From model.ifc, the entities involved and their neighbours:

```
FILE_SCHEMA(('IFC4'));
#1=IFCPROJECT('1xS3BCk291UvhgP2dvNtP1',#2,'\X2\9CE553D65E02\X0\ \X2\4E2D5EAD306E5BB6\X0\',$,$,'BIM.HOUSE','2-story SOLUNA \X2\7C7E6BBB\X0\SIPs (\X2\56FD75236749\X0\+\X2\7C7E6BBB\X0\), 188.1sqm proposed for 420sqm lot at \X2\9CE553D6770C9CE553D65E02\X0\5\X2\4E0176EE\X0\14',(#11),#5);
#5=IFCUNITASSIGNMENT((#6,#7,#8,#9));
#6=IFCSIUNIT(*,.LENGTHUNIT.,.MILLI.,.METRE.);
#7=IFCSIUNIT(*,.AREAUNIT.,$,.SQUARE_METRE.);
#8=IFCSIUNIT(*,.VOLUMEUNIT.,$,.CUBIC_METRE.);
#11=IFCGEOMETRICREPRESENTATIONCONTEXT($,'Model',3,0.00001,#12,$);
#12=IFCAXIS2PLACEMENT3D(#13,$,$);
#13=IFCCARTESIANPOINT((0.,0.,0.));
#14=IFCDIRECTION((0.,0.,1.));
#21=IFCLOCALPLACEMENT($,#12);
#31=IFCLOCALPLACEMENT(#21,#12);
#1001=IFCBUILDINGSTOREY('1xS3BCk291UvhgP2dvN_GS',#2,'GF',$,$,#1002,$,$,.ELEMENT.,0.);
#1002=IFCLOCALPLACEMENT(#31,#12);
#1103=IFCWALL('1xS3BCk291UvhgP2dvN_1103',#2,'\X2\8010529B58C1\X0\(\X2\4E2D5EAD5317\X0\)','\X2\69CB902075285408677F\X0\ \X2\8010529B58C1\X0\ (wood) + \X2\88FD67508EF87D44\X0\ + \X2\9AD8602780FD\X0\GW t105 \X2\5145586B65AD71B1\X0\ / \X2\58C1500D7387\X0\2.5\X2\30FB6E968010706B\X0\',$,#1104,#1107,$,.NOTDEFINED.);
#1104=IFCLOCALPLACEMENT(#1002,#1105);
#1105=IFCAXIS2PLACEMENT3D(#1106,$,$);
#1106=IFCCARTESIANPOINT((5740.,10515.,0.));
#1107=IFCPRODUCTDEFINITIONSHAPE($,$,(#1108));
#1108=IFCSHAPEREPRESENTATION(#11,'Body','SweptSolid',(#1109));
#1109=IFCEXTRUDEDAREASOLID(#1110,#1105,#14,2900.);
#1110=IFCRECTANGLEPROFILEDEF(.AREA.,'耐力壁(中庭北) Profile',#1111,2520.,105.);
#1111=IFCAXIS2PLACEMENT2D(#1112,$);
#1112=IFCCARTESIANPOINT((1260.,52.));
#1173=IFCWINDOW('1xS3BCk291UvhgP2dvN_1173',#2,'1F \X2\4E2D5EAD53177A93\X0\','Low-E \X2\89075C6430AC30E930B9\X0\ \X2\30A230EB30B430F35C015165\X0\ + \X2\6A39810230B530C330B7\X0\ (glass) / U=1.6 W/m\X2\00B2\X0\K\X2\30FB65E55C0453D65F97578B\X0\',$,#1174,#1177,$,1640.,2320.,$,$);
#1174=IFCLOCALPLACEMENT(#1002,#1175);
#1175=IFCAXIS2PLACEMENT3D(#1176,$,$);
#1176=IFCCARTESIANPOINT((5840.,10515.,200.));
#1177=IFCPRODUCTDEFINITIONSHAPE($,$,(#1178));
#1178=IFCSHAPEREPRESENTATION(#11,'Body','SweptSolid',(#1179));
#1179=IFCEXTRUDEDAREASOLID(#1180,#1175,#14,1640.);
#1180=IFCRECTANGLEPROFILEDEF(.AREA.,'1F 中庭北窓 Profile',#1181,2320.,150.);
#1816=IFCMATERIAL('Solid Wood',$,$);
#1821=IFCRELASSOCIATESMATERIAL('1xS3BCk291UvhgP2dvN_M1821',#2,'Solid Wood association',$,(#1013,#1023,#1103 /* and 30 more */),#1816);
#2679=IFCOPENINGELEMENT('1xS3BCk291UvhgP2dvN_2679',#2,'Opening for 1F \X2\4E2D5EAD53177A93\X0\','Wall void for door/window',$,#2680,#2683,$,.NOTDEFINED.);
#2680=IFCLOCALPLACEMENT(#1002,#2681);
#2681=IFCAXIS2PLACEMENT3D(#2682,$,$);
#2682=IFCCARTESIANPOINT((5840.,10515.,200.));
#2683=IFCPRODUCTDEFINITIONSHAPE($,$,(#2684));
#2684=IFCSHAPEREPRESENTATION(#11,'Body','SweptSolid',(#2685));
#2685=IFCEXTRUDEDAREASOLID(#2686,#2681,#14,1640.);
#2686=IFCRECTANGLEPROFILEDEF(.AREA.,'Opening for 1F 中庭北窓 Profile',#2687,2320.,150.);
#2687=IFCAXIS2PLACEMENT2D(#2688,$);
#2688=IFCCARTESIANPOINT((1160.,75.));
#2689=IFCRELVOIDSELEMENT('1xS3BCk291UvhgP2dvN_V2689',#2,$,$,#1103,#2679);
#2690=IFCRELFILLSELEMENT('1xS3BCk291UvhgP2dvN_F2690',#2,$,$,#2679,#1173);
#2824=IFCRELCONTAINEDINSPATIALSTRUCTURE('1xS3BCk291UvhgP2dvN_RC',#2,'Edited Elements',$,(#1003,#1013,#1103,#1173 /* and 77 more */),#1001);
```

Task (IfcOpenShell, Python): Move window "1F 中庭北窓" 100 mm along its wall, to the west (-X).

```python
import ifcopenshell
import ifcopenshell.api.geometry
import ifcopenshell.util.placement

model = ifcopenshell.open("model.ifc")

window = model.by_guid("1xS3BCk291UvhgP2dvN_1173")
opening = window.FillsVoids[0].RelatingOpeningElement
wall = opening.VoidsElements[0].RelatingBuildingElement

wall_matrix = ifcopenshell.util.placement.get_local_placement(wall.ObjectPlacement)
shift = wall_matrix[:3, 0] * -100.0
before = ifcopenshell.util.placement.get_local_placement(window.ObjectPlacement)[:3, 3].copy()

# The window is not placed relative to its opening, so move both.
for product in (opening, window):
    matrix = ifcopenshell.util.placement.get_local_placement(product.ObjectPlacement)
    matrix[:3, 3] += shift
    ifcopenshell.api.geometry.edit_object_placement(model, product=product, matrix=matrix, is_si=False)

after = ifcopenshell.util.placement.get_local_placement(window.ObjectPlacement)[:3, 3]
print("window moved by", (after - before).round(3) + 0.0)

model.write("model-out.ifc")
```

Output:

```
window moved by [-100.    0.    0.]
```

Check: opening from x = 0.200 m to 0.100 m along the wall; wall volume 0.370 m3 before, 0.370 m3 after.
